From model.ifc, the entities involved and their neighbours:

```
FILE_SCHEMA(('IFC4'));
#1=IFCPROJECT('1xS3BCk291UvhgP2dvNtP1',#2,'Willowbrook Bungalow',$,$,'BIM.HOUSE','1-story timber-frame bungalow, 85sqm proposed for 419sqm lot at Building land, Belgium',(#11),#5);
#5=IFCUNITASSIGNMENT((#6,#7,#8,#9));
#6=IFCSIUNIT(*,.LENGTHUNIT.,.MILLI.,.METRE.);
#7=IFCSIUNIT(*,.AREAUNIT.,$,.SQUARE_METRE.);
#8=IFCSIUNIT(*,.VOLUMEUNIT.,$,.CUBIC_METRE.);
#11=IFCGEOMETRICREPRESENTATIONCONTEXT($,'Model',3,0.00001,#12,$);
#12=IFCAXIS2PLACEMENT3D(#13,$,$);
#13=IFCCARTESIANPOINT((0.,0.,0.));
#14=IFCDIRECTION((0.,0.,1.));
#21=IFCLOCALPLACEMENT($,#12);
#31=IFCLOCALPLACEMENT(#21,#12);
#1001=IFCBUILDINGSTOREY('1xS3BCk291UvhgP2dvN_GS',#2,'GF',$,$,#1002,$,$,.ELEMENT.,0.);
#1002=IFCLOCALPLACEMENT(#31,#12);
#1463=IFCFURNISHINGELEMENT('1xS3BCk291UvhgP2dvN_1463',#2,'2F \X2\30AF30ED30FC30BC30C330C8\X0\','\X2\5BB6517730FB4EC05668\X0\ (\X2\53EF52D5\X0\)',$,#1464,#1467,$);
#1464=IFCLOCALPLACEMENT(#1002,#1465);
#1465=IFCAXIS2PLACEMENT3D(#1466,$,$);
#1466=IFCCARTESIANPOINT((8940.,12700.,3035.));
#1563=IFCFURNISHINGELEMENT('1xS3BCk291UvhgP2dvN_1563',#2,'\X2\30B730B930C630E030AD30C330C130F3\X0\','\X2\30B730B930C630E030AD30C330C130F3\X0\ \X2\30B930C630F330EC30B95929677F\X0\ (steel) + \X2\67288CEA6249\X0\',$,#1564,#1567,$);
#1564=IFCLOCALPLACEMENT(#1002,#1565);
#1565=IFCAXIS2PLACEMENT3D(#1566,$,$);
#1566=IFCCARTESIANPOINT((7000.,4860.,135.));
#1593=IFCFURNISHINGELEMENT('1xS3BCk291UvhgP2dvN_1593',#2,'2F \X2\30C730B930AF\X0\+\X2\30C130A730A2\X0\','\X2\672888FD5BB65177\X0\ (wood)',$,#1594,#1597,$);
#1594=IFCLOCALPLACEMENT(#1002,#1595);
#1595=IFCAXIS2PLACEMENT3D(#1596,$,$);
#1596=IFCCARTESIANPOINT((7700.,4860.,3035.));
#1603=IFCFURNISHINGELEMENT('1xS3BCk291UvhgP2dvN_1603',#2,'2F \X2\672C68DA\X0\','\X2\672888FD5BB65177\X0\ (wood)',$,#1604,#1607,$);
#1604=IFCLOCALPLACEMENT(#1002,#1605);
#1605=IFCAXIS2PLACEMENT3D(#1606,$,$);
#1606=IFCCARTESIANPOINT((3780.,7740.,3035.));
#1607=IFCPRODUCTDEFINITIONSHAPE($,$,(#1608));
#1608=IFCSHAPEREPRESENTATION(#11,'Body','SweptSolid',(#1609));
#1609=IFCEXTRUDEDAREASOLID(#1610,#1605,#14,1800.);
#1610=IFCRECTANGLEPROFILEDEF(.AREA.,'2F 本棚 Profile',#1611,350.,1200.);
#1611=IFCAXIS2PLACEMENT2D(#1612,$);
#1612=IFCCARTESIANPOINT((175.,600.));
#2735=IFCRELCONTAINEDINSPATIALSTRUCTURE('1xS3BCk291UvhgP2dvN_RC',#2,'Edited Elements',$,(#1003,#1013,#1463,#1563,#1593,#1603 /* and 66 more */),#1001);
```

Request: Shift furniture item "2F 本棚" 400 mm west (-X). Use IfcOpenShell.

```python
import ifcopenshell
import ifcopenshell.api.geometry
import ifcopenshell.util.placement
import ifcopenshell.util.unit

model = ifcopenshell.open("model.ifc")
unit_scale = ifcopenshell.util.unit.calculate_unit_scale(model)

item = model.by_guid("1xS3BCk291UvhgP2dvN_1603")
matrix = ifcopenshell.util.placement.get_local_placement(item.ObjectPlacement)
matrix[0, 3] -= 0.4 / unit_scale
ifcopenshell.api.geometry.edit_object_placement(model, product=item, matrix=matrix, is_si=False)

print(ifcopenshell.util.placement.get_local_placement(item.ObjectPlacement).round(3) + 0.0)

model.write("model_updated.ifc")
```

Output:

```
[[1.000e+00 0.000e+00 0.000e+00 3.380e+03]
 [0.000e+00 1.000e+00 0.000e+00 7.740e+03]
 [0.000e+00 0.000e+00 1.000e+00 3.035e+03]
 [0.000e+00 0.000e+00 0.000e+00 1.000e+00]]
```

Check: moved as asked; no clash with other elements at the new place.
